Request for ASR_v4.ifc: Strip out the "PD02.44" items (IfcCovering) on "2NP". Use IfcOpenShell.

First a look at what the model holds.

```python
import ifcopenshell
import ifcopenshell.util.element

model = ifcopenshell.open("ASR_v4.ifc")
print(model.schema)
storey = next(s for s in model.by_type("IfcBuildingStorey") if s.Name == "2NP")
coverings = [e for e in ifcopenshell.util.element.get_decomposition(storey) if e.is_a("IfcCovering")]
seen = {}
for e in coverings:
    element_type = ifcopenshell.util.element.get_type(e)
    name = element_type.Name if element_type not in (None, e) else None
    seen[name] = seen.get(name, 0) + 1
for name, count in sorted(seen.items(), key=str):
    print(count, "x", name)
```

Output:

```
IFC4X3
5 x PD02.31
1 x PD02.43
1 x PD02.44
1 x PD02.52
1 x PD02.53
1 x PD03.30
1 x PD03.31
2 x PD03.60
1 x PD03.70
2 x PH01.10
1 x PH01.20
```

```python
import ifcopenshell
import ifcopenshell.api.root
import ifcopenshell.util.element

model = ifcopenshell.open("ASR_v4.ifc")

storey = next(s for s in model.by_type("IfcBuildingStorey") if s.Name == "2NP")
coverings = [e for e in ifcopenshell.util.element.get_decomposition(storey) if e.is_a("IfcCovering")]
targets = [e for e in coverings if (t := ifcopenshell.util.element.get_type(e)) not in (None, e) and t.Name == "PD02.44"]

for e in targets:
    ifcopenshell.api.root.remove_product(model, product=e)
print(len(targets), "removed")

model.write("ASR_v4_updated.ifc")
```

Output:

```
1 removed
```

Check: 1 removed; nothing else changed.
